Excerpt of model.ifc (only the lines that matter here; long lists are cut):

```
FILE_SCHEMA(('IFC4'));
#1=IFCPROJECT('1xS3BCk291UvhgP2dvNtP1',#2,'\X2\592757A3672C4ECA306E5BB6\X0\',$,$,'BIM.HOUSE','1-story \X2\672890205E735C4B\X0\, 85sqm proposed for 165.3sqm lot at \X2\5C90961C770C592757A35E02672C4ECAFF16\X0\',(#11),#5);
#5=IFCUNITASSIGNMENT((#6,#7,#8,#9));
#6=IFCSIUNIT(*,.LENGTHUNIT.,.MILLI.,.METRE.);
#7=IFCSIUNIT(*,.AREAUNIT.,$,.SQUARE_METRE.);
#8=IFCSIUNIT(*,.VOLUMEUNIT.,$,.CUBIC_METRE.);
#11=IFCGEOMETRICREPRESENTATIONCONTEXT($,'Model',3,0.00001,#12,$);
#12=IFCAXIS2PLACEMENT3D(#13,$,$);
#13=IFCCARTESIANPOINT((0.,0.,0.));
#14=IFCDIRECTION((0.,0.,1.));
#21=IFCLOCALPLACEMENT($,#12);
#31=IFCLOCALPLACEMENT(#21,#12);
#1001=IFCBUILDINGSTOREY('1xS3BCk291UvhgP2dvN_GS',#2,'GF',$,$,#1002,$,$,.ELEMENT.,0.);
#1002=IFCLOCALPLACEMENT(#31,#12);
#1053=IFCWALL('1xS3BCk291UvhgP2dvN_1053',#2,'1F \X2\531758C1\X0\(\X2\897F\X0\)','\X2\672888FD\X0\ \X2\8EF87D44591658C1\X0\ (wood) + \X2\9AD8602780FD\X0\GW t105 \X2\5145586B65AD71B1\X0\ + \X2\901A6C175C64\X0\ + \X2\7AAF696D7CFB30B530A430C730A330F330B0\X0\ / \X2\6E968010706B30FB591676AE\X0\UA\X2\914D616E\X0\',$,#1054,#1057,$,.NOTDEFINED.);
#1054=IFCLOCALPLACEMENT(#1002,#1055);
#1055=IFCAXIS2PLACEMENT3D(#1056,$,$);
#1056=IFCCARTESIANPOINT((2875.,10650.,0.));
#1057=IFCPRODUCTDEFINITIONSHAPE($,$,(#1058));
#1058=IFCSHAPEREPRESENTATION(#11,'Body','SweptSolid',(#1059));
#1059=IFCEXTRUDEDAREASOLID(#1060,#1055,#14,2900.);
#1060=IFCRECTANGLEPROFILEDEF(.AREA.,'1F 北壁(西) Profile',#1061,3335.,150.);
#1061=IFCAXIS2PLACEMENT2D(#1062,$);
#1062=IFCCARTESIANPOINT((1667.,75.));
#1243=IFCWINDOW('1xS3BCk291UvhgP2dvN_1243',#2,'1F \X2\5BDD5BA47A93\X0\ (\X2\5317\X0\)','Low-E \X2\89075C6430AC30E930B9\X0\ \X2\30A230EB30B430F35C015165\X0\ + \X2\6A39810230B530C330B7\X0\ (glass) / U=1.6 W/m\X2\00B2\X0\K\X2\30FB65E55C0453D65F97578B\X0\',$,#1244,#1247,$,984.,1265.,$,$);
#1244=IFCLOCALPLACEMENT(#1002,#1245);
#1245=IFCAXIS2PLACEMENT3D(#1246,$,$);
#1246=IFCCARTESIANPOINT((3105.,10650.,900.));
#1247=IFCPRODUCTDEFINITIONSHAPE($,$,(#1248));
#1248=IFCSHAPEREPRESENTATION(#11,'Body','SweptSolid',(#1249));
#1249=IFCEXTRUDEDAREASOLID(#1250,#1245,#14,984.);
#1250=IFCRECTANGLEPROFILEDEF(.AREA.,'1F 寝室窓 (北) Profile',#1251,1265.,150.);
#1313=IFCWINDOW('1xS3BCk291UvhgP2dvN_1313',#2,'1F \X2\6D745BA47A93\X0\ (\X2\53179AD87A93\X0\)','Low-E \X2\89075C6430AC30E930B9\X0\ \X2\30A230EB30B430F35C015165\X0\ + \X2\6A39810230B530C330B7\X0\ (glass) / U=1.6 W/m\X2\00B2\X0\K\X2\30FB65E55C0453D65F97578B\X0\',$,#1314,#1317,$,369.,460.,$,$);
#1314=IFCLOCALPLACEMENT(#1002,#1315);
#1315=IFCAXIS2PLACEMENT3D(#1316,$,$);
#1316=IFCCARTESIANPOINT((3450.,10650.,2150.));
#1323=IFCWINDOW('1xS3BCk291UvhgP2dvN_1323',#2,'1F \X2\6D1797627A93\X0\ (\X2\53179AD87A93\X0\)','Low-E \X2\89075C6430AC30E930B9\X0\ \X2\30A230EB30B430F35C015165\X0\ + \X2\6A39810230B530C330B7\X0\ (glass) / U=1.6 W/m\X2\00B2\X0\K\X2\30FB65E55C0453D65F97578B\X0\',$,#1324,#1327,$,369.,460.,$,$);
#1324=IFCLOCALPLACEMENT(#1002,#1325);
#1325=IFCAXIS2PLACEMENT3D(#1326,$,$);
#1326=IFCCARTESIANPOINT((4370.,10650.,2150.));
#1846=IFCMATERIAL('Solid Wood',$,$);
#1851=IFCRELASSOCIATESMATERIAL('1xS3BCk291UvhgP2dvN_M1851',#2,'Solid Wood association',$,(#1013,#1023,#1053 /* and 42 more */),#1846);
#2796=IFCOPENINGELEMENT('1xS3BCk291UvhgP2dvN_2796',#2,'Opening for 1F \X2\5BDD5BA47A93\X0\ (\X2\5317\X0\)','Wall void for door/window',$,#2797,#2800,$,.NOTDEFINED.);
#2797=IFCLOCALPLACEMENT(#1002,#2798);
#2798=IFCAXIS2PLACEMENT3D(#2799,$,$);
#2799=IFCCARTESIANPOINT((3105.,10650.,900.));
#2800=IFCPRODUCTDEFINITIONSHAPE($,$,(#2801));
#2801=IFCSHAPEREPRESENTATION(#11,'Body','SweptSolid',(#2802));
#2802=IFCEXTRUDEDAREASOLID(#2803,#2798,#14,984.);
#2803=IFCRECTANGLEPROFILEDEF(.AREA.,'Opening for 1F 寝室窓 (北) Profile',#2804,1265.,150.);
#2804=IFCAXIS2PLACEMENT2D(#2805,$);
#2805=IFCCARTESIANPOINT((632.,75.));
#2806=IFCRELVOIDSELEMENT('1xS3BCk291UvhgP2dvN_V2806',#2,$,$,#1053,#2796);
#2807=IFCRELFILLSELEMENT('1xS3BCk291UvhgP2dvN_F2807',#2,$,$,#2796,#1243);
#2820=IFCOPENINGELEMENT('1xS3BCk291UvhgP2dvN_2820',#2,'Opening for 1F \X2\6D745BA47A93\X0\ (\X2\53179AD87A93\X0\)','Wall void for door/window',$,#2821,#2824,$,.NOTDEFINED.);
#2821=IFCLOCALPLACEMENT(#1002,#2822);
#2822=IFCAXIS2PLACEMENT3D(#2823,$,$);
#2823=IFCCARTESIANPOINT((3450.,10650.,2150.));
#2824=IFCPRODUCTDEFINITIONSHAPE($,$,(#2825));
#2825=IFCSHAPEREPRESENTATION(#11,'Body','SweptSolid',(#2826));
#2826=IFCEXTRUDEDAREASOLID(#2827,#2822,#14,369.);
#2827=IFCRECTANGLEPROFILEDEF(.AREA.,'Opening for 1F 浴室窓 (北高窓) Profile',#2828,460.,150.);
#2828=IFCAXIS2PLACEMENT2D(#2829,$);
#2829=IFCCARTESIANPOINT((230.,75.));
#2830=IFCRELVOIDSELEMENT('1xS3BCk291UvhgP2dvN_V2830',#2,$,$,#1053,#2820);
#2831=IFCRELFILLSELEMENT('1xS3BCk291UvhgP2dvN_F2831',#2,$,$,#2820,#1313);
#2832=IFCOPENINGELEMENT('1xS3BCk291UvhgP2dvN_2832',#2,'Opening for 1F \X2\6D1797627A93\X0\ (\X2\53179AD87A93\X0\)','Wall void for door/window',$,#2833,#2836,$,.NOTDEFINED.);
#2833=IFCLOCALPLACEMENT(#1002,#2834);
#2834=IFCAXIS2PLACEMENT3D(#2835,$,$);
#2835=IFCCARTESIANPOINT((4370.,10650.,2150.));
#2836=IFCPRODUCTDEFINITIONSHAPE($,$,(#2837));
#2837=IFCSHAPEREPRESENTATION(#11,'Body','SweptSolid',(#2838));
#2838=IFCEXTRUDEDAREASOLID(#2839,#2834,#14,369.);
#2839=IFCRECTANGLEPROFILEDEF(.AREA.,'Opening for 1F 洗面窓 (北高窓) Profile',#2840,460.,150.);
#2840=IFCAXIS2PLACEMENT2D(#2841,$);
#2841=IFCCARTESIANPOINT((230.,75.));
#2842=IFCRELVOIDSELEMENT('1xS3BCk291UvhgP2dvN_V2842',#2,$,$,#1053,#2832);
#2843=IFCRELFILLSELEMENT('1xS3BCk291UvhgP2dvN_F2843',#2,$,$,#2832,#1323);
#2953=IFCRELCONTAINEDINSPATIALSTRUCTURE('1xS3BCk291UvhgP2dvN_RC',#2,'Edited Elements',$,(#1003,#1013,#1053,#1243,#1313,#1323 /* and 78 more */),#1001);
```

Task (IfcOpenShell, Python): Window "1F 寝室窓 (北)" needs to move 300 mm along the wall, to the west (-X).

```python
import ifcopenshell
import ifcopenshell.api.geometry
import ifcopenshell.util.placement
import ifcopenshell.util.unit

model = ifcopenshell.open("model.ifc")
unit_scale = ifcopenshell.util.unit.calculate_unit_scale(model)

window = model.by_guid("1xS3BCk291UvhgP2dvN_1243")
opening = window.FillsVoids[0].RelatingOpeningElement
wall = opening.VoidsElements[0].RelatingBuildingElement

wall_matrix = ifcopenshell.util.placement.get_local_placement(wall.ObjectPlacement)
shift = wall_matrix[:3, 0] * -0.3 / unit_scale
before = ifcopenshell.util.placement.get_local_placement(window.ObjectPlacement)[:3, 3].copy()

# The window is not placed relative to its opening, so move both.
for product in (opening, window):
    matrix = ifcopenshell.util.placement.get_local_placement(product.ObjectPlacement)
    matrix[:3, 3] += shift
    ifcopenshell.api.geometry.edit_object_placement(model, product=product, matrix=matrix, is_si=False)

after = ifcopenshell.util.placement.get_local_placement(window.ObjectPlacement)[:3, 3]
print("window moved by", (after - before).round(3) + 0.0)

model.write("model_rev.ifc")
```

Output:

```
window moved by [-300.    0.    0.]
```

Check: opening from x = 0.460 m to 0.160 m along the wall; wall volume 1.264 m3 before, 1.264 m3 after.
